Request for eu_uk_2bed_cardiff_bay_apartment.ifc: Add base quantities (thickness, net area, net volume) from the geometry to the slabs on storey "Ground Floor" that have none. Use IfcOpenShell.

First a look at what the model holds.

```python
import ifcopenshell
import ifcopenshell.util.element
import ifcopenshell.util.unit

model = ifcopenshell.open("eu_uk_2bed_cardiff_bay_apartment.ifc")
print(model.schema)
for unit_type in ("LENGTHUNIT", "AREAUNIT", "VOLUMEUNIT"):
    print(unit_type, ifcopenshell.util.unit.calculate_unit_scale(model, unit_type))
storey = next(s for s in model.by_type("IfcBuildingStorey") if s.Name == "Ground Floor")
slabs = [e for e in ifcopenshell.util.element.get_decomposition(storey) if e.is_a("IfcSlab")]
for e in sorted(slabs, key=lambda e: e.id()):
    print(e.id(), e.is_a(), e.Name, list(ifcopenshell.util.element.get_psets(e, qtos_only=True)), sep=" | ")
```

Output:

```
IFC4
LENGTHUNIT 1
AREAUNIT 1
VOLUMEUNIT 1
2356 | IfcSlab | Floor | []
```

```python
import ifcopenshell
import ifcopenshell.api.pset
import ifcopenshell.geom
import ifcopenshell.util.element
import ifcopenshell.util.shape
import ifcopenshell.util.unit

model = ifcopenshell.open("eu_uk_2bed_cardiff_bay_apartment.ifc")
unit_scale = ifcopenshell.util.unit.calculate_unit_scale(model)
area_scale = ifcopenshell.util.unit.calculate_unit_scale(model, "AREAUNIT")
volume_scale = ifcopenshell.util.unit.calculate_unit_scale(model, "VOLUMEUNIT")
settings = ifcopenshell.geom.settings()

storey = next(s for s in model.by_type("IfcBuildingStorey") if s.Name == "Ground Floor")
slabs = [e for e in ifcopenshell.util.element.get_decomposition(storey) if e.is_a("IfcSlab")]

for e in sorted(slabs, key=lambda e: e.id()):
    if ifcopenshell.util.element.get_psets(e, qtos_only=True, should_inherit=False):
        continue
    # Geometry comes back in metres, in the element's own axes.
    shape = ifcopenshell.geom.create_shape(settings, e)
    values = {
        "Width": ifcopenshell.util.shape.get_z(shape.geometry) / unit_scale,
        "NetArea": ifcopenshell.util.shape.get_footprint_area(shape.geometry) / area_scale,
        "NetVolume": ifcopenshell.util.shape.get_volume(shape.geometry) / volume_scale,
    }
    qto = ifcopenshell.api.pset.add_qto(model, product=e, name="Qto_SlabBaseQuantities")
    ifcopenshell.api.pset.edit_qto(model, qto=qto, properties=values)
    print(e.id(), {k: round(v, 3) for k, v in values.items()})

model.write("eu_uk_2bed_cardiff_bay_apartment_edited.ifc")
```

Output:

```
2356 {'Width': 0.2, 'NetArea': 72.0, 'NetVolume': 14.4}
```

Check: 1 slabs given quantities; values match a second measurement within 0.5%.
